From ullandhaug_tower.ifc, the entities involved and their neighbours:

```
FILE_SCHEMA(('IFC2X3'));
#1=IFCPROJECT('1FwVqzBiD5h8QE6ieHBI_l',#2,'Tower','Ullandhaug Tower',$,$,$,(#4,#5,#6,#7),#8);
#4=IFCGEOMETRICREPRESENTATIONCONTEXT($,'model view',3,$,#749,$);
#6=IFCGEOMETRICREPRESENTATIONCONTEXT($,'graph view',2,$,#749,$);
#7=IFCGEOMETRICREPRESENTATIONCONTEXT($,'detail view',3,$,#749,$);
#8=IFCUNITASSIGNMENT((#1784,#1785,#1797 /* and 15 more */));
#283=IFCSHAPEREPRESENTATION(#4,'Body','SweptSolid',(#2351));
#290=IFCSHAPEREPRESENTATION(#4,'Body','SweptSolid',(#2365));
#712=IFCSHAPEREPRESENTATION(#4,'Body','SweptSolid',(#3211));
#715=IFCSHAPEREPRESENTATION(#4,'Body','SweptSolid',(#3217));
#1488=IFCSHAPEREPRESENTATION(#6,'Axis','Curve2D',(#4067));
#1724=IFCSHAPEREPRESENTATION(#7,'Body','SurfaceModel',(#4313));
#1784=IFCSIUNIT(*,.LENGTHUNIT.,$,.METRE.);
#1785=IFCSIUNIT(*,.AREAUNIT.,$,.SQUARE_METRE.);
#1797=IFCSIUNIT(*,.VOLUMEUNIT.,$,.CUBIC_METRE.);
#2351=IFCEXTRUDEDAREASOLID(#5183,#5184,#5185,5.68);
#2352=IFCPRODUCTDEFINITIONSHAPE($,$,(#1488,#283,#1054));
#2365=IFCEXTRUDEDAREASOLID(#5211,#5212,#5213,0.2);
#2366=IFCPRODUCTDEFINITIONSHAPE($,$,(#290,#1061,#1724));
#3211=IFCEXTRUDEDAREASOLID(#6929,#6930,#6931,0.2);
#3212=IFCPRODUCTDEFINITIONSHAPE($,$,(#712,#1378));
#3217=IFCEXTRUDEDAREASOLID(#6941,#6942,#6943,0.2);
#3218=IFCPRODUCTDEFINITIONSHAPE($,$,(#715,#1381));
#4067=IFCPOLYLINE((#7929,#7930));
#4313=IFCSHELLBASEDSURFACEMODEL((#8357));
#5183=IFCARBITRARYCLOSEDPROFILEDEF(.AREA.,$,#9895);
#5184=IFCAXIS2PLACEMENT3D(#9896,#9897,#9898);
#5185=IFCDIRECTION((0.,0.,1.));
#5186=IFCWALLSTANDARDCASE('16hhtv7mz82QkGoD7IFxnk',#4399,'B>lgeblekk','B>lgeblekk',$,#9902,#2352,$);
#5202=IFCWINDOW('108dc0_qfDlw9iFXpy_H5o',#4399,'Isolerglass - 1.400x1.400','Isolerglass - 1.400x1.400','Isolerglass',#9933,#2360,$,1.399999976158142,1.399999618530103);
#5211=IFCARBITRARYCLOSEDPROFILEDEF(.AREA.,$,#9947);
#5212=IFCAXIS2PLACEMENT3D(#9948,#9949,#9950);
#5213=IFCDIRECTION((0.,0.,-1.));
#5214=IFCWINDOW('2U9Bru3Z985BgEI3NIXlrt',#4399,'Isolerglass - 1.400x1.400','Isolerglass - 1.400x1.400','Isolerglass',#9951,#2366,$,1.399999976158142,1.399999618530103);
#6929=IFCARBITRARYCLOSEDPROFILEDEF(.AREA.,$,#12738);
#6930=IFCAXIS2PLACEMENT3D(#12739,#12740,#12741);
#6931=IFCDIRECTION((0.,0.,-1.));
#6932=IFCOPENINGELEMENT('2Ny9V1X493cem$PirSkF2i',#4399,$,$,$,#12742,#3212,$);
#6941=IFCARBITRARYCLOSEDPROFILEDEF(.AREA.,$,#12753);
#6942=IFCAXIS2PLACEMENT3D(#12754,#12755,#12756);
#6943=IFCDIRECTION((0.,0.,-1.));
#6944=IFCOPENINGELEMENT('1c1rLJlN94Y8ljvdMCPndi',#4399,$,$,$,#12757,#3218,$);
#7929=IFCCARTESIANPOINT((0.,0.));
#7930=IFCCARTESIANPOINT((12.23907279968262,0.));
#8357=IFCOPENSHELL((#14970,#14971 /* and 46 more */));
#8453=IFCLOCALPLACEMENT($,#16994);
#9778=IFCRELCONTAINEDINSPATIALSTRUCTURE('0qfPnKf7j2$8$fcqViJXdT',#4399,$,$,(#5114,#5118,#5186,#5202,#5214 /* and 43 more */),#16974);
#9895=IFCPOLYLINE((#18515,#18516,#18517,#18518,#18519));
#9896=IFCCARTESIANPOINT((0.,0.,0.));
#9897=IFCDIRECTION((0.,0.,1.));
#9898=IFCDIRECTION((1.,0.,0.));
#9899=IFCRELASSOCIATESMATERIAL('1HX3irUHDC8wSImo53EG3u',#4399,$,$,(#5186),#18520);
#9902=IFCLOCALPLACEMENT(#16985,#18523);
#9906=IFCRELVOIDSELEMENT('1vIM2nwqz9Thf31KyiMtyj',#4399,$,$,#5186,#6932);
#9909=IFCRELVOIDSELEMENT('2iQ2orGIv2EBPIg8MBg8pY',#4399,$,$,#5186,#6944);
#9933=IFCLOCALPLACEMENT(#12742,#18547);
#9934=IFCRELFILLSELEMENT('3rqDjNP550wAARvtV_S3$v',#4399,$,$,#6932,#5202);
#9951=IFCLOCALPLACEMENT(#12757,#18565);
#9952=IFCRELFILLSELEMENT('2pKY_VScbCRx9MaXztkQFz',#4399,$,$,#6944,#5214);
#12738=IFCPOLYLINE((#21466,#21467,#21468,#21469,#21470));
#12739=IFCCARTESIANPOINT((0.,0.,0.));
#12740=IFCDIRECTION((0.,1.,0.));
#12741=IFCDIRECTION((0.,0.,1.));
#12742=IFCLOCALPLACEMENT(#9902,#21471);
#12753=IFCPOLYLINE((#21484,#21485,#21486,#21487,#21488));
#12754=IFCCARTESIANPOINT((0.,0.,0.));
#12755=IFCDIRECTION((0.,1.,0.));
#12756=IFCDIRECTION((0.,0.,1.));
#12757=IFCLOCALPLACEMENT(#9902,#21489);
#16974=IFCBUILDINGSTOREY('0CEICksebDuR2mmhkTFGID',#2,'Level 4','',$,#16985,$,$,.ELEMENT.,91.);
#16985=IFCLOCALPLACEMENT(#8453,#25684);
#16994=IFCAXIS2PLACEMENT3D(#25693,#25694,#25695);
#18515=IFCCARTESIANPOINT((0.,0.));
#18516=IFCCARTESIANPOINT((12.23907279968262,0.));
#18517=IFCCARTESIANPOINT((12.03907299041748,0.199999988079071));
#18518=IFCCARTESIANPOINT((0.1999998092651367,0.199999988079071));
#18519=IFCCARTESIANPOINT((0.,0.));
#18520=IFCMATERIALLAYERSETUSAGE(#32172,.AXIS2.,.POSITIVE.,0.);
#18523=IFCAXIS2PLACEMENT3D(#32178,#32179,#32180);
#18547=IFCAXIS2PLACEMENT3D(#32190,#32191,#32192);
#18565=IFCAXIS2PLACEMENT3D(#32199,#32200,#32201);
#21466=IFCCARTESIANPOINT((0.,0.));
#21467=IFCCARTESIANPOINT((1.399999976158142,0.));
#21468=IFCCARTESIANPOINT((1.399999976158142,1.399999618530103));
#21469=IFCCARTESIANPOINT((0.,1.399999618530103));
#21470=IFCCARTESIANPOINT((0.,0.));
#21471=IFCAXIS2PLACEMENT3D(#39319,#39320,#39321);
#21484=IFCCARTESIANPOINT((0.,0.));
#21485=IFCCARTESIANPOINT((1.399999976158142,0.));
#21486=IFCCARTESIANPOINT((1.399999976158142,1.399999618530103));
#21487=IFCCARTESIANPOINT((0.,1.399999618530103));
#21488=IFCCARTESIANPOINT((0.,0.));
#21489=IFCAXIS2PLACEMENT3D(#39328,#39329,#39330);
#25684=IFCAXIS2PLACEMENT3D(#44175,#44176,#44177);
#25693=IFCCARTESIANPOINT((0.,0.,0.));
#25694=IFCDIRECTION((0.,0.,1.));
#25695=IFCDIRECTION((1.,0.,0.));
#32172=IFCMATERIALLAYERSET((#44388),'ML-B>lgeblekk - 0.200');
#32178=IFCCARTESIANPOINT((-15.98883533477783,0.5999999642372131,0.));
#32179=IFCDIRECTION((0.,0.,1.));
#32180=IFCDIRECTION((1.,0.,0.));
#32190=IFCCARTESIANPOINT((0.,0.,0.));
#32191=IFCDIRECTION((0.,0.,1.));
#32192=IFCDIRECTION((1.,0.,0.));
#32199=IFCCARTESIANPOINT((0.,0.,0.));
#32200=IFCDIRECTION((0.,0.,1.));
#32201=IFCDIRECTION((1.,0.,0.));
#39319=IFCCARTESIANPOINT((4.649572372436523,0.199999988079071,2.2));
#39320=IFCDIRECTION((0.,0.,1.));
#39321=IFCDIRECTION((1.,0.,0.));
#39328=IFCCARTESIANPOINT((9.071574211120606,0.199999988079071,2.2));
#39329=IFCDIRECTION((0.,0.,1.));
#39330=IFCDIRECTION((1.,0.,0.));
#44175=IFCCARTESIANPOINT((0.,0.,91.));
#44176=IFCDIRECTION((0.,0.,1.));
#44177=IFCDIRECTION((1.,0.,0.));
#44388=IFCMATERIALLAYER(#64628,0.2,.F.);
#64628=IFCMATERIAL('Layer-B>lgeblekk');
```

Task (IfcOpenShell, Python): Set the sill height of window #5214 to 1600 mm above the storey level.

```python
import numpy as np
import ifcopenshell
import ifcopenshell.api.geometry
import ifcopenshell.geom
import ifcopenshell.util.element
import ifcopenshell.util.placement
import ifcopenshell.util.shape
import ifcopenshell.util.unit

model = ifcopenshell.open("ullandhaug_tower.ifc")
unit_scale = ifcopenshell.util.unit.calculate_unit_scale(model)

window = model.by_guid("2U9Bru3Z985BgEI3NIXlrt")
opening = window.FillsVoids[0].RelatingOpeningElement
storey = ifcopenshell.util.element.get_container(window, ifc_class="IfcBuildingStorey")
level = ifcopenshell.util.placement.get_local_placement(storey.ObjectPlacement)[2, 3]

# The opening's origin need not be at the sill, so measure its lowest point.
shape = ifcopenshell.geom.create_shape(ifcopenshell.geom.settings(), opening)
bottom = ifcopenshell.util.shape.get_shape_bottom_elevation(shape, shape.geometry) / unit_scale
dz = level + 1.6 - bottom

shift = np.array([0.0, 0.0, dz])
# The window is placed relative to its opening, so it follows when the opening moves.
matrix = ifcopenshell.util.placement.get_local_placement(opening.ObjectPlacement)
matrix[:3, 3] += shift
ifcopenshell.api.geometry.edit_object_placement(
    model, product=opening, matrix=matrix, is_si=False, should_transform_children=True
)

print(f"moved by {dz * unit_scale:+.3f} m")

model.write("ullandhaug_tower_updated.ifc")
```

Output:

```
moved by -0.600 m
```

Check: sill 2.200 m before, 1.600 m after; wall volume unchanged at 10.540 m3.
